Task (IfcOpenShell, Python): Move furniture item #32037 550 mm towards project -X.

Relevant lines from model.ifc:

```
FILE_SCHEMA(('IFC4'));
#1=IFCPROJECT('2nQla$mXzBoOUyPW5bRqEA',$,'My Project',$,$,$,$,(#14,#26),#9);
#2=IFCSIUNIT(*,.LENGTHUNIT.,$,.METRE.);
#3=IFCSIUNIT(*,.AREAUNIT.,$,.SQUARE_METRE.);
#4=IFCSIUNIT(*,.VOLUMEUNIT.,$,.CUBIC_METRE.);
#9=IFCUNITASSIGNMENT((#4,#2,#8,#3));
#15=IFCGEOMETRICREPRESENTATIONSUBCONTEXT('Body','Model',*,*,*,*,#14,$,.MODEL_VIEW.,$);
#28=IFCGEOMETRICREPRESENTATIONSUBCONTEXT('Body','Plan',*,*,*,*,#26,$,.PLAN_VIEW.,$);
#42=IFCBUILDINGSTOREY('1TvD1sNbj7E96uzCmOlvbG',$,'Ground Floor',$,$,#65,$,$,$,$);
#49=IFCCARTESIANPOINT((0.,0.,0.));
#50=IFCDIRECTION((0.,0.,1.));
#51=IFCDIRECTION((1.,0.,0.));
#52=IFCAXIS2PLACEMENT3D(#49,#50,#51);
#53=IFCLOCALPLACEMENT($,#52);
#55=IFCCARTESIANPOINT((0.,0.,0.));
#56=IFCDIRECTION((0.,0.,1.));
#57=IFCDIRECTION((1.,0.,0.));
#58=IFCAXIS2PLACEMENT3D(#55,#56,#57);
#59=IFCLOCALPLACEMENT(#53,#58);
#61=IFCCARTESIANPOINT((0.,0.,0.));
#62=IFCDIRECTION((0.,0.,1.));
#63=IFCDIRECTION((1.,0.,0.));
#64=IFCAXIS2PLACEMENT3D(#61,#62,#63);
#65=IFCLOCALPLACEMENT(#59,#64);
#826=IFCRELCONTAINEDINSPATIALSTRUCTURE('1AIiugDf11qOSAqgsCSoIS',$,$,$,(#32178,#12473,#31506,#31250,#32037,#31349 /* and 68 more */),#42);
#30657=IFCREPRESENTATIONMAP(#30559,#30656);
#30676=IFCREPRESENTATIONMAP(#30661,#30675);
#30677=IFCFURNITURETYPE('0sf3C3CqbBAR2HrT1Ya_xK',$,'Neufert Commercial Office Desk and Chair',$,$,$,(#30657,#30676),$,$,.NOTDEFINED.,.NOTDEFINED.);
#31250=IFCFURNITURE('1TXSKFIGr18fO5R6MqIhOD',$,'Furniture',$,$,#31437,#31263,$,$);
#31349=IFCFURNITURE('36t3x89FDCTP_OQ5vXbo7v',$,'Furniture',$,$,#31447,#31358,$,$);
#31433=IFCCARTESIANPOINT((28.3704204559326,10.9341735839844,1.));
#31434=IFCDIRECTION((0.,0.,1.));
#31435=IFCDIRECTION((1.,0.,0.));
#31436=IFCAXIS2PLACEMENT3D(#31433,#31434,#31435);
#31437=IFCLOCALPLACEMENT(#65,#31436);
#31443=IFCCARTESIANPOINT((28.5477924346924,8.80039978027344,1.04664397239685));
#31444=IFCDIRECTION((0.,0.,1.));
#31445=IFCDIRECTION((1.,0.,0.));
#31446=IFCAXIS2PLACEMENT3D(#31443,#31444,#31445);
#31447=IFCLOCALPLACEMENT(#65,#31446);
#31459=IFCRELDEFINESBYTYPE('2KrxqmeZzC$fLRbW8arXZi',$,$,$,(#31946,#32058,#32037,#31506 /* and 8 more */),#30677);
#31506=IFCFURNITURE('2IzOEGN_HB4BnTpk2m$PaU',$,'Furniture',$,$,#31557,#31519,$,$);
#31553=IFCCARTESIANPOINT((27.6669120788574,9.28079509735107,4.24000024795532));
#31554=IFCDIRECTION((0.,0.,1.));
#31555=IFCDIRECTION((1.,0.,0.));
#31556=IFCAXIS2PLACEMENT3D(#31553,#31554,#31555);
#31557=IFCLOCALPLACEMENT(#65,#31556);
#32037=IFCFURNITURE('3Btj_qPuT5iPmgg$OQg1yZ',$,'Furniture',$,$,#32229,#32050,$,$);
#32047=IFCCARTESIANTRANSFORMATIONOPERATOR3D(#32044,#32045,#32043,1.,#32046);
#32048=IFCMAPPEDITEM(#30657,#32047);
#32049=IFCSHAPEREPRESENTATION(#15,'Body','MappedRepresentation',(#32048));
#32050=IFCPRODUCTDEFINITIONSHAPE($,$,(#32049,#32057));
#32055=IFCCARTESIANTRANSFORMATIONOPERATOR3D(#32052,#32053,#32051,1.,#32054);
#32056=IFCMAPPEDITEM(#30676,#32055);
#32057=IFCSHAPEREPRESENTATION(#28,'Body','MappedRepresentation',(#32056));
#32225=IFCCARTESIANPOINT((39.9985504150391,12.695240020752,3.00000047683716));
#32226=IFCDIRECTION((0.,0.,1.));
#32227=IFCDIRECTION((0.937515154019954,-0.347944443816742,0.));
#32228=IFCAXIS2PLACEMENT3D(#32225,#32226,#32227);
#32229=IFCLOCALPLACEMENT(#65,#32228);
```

```python
import ifcopenshell
import ifcopenshell.api.geometry
import ifcopenshell.util.placement
import ifcopenshell.util.unit

model = ifcopenshell.open("model.ifc")
unit_scale = ifcopenshell.util.unit.calculate_unit_scale(model)

item = model.by_guid("3Btj_qPuT5iPmgg$OQg1yZ")
matrix = ifcopenshell.util.placement.get_local_placement(item.ObjectPlacement)
matrix[0, 3] -= 0.55 / unit_scale
ifcopenshell.api.geometry.edit_object_placement(model, product=item, matrix=matrix, is_si=False)

print(ifcopenshell.util.placement.get_local_placement(item.ObjectPlacement).round(3) + 0.0)

model.write("model_rev.ifc")
```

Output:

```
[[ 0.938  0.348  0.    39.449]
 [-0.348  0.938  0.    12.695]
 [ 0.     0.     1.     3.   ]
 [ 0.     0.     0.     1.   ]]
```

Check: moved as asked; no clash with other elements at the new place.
